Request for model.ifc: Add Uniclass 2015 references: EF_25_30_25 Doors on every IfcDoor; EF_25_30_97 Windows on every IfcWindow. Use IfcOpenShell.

First a look at what the model holds.

```python
import ifcopenshell

model = ifcopenshell.open("model.ifc")
print(model.schema)
print("classifications:", [c.Name for c in model.by_type("IfcClassification")])
for ifc_class in ("IfcDoor", "IfcRoof", "IfcStair", "IfcWall", "IfcWindow"):
    print(ifc_class, len(model.by_type(ifc_class)))
```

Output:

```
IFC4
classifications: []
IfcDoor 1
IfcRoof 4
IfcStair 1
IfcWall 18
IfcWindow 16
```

```python
import ifcopenshell
import ifcopenshell.api.classification

model = ifcopenshell.open("model.ifc")

system = ifcopenshell.api.classification.add_classification(model, classification="Uniclass 2015")

codes = {
    "IfcDoor": ("EF_25_30_25", "Doors"),
    "IfcWindow": ("EF_25_30_97", "Windows"),
}
for ifc_class, (code, name) in codes.items():
    products = model.by_type(ifc_class)
    ifcopenshell.api.classification.add_reference(
        model, products=products, classification=system, identification=code, name=name
    )
    print(code, len(products))

model.write("model-out.ifc")
```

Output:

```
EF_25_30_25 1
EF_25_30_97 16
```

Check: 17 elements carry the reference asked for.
